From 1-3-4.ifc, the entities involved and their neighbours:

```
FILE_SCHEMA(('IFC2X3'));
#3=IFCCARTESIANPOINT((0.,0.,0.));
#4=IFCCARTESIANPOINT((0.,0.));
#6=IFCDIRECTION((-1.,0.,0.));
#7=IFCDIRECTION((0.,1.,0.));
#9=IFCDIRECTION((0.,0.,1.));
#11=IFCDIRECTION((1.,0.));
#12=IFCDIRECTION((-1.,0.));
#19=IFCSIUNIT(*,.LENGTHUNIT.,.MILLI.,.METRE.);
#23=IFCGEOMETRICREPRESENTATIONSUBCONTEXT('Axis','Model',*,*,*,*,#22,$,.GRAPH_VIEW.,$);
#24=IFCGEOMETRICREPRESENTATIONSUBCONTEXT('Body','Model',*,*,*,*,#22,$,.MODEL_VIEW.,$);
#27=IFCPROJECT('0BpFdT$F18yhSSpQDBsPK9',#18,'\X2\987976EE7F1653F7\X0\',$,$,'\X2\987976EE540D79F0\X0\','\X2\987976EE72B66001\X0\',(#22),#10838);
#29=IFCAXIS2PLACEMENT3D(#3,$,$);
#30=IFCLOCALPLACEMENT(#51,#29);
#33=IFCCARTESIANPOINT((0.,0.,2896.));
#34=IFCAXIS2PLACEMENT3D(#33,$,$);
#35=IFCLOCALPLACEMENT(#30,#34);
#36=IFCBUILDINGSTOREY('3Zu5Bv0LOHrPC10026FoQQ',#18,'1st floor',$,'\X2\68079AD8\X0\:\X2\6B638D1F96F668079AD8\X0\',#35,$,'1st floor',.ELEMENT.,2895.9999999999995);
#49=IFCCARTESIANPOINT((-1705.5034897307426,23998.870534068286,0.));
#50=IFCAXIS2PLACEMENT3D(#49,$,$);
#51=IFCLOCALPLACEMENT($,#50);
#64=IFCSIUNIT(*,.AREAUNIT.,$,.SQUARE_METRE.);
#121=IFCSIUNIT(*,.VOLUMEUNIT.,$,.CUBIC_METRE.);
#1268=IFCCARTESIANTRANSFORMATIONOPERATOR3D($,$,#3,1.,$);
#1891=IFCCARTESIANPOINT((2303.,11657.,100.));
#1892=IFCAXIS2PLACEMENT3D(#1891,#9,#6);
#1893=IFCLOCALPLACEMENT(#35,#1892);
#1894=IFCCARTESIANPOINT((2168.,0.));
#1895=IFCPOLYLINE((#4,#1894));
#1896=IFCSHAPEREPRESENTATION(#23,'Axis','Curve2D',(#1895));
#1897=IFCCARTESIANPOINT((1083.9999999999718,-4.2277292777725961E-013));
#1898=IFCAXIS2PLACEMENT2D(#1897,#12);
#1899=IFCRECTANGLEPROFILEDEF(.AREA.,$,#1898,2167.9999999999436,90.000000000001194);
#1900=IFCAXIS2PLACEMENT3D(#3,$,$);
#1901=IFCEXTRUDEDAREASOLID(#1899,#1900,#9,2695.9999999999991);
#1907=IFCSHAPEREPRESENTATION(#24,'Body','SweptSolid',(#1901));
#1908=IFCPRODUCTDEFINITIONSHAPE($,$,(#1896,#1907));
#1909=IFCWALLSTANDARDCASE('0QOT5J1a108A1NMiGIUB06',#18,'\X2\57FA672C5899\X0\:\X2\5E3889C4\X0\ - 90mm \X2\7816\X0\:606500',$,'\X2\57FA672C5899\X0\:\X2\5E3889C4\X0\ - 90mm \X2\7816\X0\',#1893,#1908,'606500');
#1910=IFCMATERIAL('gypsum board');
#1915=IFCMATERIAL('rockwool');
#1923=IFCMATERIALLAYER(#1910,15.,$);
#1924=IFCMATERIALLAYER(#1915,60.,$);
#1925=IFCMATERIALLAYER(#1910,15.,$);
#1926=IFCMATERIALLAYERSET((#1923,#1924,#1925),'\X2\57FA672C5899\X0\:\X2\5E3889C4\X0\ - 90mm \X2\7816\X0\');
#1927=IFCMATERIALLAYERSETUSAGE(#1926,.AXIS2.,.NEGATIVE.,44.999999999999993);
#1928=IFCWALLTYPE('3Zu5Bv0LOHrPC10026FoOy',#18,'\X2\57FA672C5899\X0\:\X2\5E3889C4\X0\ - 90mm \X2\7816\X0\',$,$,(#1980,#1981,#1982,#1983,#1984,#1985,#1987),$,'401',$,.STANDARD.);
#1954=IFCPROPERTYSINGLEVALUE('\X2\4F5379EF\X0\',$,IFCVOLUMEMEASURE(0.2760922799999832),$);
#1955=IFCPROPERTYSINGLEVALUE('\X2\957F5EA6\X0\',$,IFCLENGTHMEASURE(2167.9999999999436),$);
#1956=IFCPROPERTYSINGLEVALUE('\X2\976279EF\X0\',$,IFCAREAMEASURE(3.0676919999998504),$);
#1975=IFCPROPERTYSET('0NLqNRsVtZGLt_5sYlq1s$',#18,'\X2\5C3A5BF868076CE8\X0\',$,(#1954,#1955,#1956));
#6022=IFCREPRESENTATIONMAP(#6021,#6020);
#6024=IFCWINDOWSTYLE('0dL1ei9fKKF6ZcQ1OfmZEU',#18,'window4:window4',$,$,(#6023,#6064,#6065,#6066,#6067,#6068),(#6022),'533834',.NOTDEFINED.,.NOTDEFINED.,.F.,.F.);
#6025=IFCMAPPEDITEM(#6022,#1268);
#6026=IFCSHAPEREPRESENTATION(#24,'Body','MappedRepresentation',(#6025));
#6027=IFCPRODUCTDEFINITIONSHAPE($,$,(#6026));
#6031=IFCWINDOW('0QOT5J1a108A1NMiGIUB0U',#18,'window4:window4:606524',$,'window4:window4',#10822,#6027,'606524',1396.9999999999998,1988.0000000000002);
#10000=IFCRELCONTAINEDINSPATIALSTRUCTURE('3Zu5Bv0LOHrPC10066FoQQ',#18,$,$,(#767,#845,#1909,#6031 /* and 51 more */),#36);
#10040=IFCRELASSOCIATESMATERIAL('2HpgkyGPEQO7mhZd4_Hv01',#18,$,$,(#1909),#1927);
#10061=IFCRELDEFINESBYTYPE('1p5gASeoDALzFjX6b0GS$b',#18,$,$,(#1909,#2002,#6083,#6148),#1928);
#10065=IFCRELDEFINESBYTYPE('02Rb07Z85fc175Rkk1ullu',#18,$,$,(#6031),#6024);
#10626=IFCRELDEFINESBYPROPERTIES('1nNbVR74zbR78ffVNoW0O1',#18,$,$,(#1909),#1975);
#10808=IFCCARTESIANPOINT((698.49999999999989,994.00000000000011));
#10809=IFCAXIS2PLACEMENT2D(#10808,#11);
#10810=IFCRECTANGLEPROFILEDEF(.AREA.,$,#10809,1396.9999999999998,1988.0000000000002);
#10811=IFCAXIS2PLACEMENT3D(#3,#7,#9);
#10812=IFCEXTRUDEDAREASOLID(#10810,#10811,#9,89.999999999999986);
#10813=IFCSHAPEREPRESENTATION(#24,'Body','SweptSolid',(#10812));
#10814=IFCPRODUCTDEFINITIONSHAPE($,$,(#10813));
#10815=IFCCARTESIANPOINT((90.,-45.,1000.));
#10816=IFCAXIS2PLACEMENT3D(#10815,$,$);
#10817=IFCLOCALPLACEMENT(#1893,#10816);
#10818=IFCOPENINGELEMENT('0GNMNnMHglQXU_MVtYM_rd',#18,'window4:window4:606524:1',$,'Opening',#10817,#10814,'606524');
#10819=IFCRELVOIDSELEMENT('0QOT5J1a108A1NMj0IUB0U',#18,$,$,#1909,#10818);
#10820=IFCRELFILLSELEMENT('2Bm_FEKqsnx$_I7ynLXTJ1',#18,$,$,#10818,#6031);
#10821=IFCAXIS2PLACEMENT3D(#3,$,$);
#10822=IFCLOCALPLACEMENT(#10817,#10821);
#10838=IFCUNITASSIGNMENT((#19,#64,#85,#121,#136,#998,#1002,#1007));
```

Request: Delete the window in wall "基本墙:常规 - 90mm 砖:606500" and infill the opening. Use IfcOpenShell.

```python
import ifcopenshell
import ifcopenshell.api.feature
import ifcopenshell.api.pset
import ifcopenshell.api.root
import ifcopenshell.geom
import ifcopenshell.util.element
import ifcopenshell.util.shape
import ifcopenshell.util.unit

model = ifcopenshell.open("1-3-4.ifc")
area_scale = ifcopenshell.util.unit.calculate_unit_scale(model, "AREAUNIT")
volume_scale = ifcopenshell.util.unit.calculate_unit_scale(model, "VOLUMEUNIT")
settings = ifcopenshell.geom.settings()


def volume(element):
    """Net volume in cubic metres, openings subtracted."""
    shape = ifcopenshell.geom.create_shape(settings, element)
    return ifcopenshell.util.shape.get_volume(shape.geometry)


window = model.by_guid("0QOT5J1a108A1NMiGIUB0U")
opening = window.FillsVoids[0].RelatingOpeningElement
wall = opening.VoidsElements[0].RelatingBuildingElement
before = volume(wall)

ifcopenshell.api.root.remove_product(model, product=window)
ifcopenshell.api.feature.remove_feature(model, feature=opening)

after = volume(wall)
thickness = 0.09  # wall thickness in metres

# Update the wall's stored quantities.
pset = model.by_id(ifcopenshell.util.element.get_pset(wall, "尺寸标注", should_inherit=False)["id"])
ifcopenshell.api.pset.edit_pset(model, pset=pset, properties={
    "体积": model.create_entity("IfcVolumeMeasure", after / volume_scale),
    "面积": model.create_entity("IfcAreaMeasure", after / thickness / area_scale),
})

print(f"wall volume {before:.3f} -> {after:.3f} m3")

model.write("1-3-4-out.ifc")
```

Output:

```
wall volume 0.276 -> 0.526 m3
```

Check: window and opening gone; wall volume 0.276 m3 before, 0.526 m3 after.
